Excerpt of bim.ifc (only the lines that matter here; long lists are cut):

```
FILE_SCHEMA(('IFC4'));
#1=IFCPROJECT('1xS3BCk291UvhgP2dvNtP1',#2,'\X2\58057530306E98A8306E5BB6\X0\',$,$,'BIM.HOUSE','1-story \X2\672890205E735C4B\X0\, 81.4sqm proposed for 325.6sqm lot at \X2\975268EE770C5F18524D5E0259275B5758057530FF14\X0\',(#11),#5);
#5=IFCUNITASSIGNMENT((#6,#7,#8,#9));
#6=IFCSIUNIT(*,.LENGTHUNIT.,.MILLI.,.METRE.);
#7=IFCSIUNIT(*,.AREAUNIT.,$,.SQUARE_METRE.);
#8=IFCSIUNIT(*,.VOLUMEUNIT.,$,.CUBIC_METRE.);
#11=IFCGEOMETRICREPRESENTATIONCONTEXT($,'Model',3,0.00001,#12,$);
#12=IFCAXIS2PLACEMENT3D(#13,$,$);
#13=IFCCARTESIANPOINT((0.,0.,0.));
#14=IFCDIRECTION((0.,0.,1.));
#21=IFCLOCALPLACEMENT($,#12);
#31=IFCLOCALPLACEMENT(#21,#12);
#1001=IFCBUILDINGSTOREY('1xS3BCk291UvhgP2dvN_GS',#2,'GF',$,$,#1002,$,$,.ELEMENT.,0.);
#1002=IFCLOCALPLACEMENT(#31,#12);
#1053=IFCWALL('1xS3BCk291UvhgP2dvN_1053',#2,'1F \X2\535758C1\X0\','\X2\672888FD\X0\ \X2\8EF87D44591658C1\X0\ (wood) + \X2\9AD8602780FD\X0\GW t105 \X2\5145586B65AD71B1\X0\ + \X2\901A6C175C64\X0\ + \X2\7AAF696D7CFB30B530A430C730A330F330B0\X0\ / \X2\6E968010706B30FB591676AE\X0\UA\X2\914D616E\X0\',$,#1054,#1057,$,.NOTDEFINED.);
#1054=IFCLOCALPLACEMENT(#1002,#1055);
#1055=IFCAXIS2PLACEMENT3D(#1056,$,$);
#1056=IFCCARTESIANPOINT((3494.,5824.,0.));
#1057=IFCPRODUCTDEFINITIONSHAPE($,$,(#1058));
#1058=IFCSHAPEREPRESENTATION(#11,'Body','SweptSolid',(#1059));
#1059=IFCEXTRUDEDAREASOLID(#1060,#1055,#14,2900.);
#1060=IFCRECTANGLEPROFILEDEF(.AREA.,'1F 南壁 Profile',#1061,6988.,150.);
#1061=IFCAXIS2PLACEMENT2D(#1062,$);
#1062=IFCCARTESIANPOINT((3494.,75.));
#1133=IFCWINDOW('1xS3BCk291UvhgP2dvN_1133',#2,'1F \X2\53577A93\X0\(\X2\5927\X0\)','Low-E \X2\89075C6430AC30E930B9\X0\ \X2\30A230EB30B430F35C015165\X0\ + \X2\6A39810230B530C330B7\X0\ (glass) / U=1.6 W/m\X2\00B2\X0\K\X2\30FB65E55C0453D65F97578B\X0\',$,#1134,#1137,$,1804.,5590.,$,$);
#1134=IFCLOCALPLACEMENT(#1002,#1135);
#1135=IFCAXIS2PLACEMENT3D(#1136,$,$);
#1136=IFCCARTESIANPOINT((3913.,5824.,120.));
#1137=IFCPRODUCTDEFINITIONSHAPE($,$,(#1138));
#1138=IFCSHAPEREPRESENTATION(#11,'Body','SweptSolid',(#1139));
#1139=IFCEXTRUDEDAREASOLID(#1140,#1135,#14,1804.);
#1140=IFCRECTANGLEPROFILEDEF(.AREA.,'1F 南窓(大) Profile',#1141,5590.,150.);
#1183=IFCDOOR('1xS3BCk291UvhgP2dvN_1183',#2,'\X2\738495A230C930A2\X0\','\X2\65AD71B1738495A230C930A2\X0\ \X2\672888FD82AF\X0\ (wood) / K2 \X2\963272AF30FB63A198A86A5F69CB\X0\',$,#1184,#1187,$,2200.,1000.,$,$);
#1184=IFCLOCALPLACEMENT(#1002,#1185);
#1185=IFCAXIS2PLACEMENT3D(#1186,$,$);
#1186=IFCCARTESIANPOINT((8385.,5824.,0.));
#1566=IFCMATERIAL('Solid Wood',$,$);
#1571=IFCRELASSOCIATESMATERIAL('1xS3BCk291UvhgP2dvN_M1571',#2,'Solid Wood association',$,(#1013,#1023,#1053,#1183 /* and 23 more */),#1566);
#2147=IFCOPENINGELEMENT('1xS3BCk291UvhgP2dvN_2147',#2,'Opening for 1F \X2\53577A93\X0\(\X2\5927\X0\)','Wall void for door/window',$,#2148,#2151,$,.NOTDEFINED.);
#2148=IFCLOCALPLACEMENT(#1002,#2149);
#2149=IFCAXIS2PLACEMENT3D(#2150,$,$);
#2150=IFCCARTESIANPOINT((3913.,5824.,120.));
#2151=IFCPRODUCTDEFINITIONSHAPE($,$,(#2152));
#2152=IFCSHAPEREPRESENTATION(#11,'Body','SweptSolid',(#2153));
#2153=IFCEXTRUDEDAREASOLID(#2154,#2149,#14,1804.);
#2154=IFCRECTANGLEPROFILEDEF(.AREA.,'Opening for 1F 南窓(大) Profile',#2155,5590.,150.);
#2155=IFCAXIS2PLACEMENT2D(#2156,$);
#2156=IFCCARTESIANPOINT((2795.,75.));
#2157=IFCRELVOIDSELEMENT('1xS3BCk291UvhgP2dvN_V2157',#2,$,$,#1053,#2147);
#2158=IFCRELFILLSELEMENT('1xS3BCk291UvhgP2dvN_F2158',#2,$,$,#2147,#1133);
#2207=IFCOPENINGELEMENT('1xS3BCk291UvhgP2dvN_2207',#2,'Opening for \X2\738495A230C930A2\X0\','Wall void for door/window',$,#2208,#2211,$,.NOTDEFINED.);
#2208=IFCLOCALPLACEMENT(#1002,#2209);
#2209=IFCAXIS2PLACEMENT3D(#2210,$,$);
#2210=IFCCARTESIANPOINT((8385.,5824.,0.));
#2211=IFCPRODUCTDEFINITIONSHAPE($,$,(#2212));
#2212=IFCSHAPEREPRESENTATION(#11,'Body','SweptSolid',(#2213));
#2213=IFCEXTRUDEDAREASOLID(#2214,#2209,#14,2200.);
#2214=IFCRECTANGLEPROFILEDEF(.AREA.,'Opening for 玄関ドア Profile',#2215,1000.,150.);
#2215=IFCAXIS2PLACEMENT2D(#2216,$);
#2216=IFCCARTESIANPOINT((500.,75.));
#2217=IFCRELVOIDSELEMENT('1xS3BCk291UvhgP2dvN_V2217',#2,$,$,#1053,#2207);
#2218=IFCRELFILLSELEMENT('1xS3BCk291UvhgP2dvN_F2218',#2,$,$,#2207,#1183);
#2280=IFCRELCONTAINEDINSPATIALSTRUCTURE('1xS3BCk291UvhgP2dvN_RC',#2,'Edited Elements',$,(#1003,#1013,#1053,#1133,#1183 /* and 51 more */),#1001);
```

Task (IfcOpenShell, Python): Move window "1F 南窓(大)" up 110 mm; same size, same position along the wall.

```python
import numpy as np
import ifcopenshell
import ifcopenshell.api.geometry
import ifcopenshell.util.placement
import ifcopenshell.util.unit

model = ifcopenshell.open("bim.ifc")
unit_scale = ifcopenshell.util.unit.calculate_unit_scale(model)

window = model.by_id(1133)
opening = window.FillsVoids[0].RelatingOpeningElement
dz = 0.11 / unit_scale

shift = np.array([0.0, 0.0, dz])
# The window is not placed relative to its opening, so move both.
for product in (opening, window):
    matrix = ifcopenshell.util.placement.get_local_placement(product.ObjectPlacement)
    matrix[:3, 3] += shift
    ifcopenshell.api.geometry.edit_object_placement(model, product=product, matrix=matrix, is_si=False)

print(f"moved by {dz * unit_scale:+.3f} m")

model.write("bim-out.ifc")
```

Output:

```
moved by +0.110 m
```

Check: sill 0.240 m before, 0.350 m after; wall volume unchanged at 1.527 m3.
